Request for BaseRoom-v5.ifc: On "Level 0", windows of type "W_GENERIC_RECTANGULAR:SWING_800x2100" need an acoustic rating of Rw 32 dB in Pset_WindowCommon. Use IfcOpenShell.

First a look at what the model holds.

```python
import ifcopenshell
import ifcopenshell.util.element

model = ifcopenshell.open("BaseRoom-v5.ifc")
print(model.schema)
storey = next(s for s in model.by_type("IfcBuildingStorey") if s.Name == "Level 0")
windows = [e for e in ifcopenshell.util.element.get_decomposition(storey) if e.is_a("IfcWindow")]
seen = {}
for e in windows:
    element_type = ifcopenshell.util.element.get_type(e)
    key = (element_type.Name if element_type != e and element_type else None, ifcopenshell.util.element.get_pset(e, "Pset_WindowCommon", "AcousticRating"))
    seen[key] = seen.get(key, 0) + 1
for (name, value), count in sorted(seen.items(), key=str):
    print(count, "x", name, "|", value)
```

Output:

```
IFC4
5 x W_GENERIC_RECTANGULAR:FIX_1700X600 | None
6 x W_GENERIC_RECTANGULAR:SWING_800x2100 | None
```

```python
import ifcopenshell
import ifcopenshell.api.pset
import ifcopenshell.util.element

model = ifcopenshell.open("BaseRoom-v5.ifc")

storey = next(s for s in model.by_type("IfcBuildingStorey") if s.Name == "Level 0")
windows = [e for e in ifcopenshell.util.element.get_decomposition(storey) if e.is_a("IfcWindow")]

count = 0
for e in windows:
    element_type = ifcopenshell.util.element.get_type(e)
    if element_type in (None, e) or element_type.Name != "W_GENERIC_RECTANGULAR:SWING_800x2100":
        continue
    # add_pset returns the element's existing set when there is one.
    pset = ifcopenshell.api.pset.add_pset(model, product=e, name="Pset_WindowCommon")
    ifcopenshell.api.pset.edit_pset(model, pset=pset, properties={"AcousticRating": "Rw 32 dB"})
    count += 1

print(count, "windows updated")

model.write("BaseRoom-v5_v2.ifc")
```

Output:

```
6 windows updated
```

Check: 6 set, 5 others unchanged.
